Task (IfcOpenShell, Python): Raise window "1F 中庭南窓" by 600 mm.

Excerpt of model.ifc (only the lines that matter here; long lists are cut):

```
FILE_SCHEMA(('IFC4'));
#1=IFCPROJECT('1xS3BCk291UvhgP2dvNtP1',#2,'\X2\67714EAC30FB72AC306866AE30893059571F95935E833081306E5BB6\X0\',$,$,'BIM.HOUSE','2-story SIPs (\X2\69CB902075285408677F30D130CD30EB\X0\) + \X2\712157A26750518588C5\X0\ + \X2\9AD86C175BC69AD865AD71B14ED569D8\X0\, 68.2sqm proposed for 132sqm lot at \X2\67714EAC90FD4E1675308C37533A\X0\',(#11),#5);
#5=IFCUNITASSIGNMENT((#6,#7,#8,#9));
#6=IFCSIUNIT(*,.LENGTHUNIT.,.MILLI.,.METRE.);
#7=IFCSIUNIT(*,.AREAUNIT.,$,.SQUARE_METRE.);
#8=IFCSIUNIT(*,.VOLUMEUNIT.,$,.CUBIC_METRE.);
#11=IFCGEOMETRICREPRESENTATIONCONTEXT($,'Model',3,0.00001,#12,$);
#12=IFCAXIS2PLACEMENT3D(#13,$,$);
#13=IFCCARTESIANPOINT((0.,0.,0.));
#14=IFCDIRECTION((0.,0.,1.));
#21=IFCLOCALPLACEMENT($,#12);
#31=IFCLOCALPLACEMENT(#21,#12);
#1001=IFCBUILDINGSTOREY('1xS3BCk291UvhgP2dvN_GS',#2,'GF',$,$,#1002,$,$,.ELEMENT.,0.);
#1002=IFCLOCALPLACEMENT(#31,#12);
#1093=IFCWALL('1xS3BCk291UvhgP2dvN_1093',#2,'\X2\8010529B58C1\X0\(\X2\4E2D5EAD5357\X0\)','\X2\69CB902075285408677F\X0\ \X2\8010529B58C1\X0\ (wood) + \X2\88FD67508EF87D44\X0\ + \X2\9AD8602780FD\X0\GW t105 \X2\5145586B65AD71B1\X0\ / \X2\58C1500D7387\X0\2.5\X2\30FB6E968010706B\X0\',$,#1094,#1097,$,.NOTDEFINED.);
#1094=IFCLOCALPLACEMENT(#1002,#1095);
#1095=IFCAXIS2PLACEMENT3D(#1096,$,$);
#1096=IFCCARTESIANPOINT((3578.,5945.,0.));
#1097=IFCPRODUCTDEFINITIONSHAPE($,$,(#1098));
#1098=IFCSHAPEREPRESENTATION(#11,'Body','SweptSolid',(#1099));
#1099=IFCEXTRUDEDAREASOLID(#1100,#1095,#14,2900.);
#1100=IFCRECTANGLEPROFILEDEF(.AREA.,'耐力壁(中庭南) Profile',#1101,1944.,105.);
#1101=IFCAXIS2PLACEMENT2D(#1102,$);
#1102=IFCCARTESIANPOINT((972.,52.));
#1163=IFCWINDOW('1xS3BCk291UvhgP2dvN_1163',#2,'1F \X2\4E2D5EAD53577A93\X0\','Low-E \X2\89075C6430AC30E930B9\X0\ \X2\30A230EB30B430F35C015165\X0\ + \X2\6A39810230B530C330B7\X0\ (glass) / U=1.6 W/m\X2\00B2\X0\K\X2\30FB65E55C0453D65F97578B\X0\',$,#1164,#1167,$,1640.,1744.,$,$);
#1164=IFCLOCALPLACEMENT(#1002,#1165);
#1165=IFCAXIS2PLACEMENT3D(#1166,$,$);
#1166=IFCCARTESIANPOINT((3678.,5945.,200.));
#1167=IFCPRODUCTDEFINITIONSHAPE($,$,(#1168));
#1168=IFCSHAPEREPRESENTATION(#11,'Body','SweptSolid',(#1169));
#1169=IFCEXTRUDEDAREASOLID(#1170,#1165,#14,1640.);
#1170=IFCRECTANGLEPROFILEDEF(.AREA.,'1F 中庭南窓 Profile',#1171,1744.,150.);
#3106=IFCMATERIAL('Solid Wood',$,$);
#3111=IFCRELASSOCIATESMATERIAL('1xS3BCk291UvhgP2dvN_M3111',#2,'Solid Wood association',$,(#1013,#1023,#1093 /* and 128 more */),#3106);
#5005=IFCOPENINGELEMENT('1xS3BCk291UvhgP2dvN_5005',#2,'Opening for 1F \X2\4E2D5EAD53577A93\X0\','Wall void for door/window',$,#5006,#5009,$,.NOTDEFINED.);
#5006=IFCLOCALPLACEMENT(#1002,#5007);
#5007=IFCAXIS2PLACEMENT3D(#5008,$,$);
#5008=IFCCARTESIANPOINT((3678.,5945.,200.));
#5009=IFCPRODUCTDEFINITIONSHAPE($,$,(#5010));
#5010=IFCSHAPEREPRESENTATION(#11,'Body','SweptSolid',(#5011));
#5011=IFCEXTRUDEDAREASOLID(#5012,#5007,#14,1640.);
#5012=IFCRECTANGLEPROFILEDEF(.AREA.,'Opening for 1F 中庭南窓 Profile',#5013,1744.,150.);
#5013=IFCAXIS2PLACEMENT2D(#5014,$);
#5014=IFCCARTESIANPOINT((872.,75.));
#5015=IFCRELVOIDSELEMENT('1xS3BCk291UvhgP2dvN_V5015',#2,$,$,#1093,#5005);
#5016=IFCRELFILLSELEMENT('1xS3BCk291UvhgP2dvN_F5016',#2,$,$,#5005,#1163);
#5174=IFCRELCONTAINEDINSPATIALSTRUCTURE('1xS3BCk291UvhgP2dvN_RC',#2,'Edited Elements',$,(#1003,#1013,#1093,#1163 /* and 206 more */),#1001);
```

```python
import numpy as np
import ifcopenshell
import ifcopenshell.api.geometry
import ifcopenshell.util.placement
import ifcopenshell.util.unit

model = ifcopenshell.open("model.ifc")
unit_scale = ifcopenshell.util.unit.calculate_unit_scale(model)

window = model.by_id(1163)
opening = window.FillsVoids[0].RelatingOpeningElement
dz = 600.0

shift = np.array([0.0, 0.0, dz])
# The window is not placed relative to its opening, so move both.
for product in (opening, window):
    matrix = ifcopenshell.util.placement.get_local_placement(product.ObjectPlacement)
    matrix[:3, 3] += shift
    ifcopenshell.api.geometry.edit_object_placement(model, product=product, matrix=matrix, is_si=False)

print(f"moved by {dz * unit_scale:+.3f} m")

model.write("model_rev.ifc")
```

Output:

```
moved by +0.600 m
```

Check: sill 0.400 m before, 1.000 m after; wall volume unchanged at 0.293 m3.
